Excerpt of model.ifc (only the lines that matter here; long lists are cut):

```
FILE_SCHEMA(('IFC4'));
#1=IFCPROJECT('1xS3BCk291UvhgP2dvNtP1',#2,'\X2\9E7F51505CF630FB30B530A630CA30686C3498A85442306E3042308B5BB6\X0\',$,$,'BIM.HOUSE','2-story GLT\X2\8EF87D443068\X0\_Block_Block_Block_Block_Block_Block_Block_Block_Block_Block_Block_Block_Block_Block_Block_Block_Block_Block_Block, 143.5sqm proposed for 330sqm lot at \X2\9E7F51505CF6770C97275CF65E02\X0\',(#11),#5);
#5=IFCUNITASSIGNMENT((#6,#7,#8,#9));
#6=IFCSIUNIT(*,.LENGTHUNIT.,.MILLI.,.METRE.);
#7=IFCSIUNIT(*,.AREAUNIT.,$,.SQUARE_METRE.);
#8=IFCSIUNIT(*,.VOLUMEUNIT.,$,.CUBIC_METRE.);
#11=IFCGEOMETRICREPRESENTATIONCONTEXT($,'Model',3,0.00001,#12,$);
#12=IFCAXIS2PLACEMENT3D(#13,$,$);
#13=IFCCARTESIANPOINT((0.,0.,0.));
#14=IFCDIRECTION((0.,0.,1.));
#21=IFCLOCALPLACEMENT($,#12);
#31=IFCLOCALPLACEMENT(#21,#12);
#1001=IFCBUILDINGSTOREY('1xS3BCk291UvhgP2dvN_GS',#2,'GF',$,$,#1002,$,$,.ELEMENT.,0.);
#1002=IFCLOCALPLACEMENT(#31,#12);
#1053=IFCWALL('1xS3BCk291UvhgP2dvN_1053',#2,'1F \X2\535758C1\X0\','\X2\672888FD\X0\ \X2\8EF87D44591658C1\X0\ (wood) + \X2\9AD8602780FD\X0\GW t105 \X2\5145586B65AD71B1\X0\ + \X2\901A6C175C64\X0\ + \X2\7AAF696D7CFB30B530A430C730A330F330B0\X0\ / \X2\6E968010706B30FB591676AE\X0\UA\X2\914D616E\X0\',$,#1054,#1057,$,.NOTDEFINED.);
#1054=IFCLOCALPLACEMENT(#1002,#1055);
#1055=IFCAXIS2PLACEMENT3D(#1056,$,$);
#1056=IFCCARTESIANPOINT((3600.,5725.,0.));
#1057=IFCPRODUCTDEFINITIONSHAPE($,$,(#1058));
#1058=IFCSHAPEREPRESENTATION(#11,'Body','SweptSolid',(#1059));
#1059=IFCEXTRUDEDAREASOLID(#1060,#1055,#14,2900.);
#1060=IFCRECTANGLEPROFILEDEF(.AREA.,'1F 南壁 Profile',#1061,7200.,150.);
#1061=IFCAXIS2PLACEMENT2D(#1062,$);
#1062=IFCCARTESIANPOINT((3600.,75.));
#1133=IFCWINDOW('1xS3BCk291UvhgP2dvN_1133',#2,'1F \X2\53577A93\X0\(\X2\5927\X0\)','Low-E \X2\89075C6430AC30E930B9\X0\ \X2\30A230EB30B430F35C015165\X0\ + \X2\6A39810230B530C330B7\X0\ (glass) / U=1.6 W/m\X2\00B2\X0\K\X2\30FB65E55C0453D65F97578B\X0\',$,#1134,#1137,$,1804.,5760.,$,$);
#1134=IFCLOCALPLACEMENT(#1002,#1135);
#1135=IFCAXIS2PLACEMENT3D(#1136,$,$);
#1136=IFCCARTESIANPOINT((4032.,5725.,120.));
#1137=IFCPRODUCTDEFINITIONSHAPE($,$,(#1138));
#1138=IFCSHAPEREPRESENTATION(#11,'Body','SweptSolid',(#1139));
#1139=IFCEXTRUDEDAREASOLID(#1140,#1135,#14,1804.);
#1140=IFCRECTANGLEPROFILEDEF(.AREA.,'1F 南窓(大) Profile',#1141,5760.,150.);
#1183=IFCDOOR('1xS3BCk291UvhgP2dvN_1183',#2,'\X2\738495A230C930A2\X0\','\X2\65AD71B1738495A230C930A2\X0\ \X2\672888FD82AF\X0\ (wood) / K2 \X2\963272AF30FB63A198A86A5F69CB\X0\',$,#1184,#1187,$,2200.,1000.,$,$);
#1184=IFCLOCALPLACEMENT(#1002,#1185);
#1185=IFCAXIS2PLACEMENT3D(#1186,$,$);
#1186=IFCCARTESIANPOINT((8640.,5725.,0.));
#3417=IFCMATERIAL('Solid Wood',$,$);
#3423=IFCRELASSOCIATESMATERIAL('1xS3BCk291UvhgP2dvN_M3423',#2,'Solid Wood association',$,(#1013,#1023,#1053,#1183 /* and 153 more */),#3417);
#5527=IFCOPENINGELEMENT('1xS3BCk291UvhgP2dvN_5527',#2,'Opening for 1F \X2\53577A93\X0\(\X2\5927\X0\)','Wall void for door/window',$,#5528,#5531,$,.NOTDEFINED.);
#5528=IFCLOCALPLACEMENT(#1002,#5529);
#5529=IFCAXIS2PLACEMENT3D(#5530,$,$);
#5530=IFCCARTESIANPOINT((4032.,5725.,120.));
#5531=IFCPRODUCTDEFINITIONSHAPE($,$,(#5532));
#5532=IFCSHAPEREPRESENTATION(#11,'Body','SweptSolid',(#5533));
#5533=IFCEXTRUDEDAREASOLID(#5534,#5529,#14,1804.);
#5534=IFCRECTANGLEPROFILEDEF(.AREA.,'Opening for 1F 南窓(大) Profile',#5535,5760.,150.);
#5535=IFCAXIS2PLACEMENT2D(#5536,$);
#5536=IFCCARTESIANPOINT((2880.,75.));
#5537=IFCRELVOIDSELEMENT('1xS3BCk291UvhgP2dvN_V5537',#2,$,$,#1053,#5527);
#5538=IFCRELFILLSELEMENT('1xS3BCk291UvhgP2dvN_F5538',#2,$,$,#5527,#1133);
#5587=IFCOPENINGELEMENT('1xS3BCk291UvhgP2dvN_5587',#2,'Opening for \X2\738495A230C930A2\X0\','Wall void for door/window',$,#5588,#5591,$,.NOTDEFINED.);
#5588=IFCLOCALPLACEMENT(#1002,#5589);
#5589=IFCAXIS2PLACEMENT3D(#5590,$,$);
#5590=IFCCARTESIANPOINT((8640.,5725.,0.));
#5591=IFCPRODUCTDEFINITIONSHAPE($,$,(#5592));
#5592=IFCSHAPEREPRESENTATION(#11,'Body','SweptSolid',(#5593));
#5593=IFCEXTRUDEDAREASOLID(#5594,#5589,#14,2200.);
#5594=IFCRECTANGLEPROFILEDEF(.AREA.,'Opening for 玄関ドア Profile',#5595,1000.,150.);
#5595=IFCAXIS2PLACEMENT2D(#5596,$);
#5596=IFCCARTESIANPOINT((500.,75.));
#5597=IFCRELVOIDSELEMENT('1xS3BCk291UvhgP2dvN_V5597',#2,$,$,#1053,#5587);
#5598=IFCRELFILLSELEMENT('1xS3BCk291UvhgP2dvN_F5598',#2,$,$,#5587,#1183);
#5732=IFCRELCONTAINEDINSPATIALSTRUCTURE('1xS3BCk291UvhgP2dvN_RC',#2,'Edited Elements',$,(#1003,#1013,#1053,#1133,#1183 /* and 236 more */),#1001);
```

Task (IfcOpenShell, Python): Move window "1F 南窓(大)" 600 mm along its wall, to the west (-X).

```python
import ifcopenshell
import ifcopenshell.api.geometry
import ifcopenshell.util.placement
import ifcopenshell.util.unit

model = ifcopenshell.open("model.ifc")
unit_scale = ifcopenshell.util.unit.calculate_unit_scale(model)

window = model.by_id(1133)
opening = window.FillsVoids[0].RelatingOpeningElement
wall = opening.VoidsElements[0].RelatingBuildingElement

wall_matrix = ifcopenshell.util.placement.get_local_placement(wall.ObjectPlacement)
shift = wall_matrix[:3, 0] * -0.6 / unit_scale
before = ifcopenshell.util.placement.get_local_placement(window.ObjectPlacement)[:3, 3].copy()

# The window is not placed relative to its opening, so move both.
for product in (opening, window):
    matrix = ifcopenshell.util.placement.get_local_placement(product.ObjectPlacement)
    matrix[:3, 3] += shift
    ifcopenshell.api.geometry.edit_object_placement(model, product=product, matrix=matrix, is_si=False)

after = ifcopenshell.util.placement.get_local_placement(window.ObjectPlacement)[:3, 3]
print("window moved by", (after - before).round(3) + 0.0)

model.write("model-out.ifc")
```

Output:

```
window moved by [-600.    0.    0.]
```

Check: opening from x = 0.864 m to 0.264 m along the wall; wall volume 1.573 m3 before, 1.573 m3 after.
